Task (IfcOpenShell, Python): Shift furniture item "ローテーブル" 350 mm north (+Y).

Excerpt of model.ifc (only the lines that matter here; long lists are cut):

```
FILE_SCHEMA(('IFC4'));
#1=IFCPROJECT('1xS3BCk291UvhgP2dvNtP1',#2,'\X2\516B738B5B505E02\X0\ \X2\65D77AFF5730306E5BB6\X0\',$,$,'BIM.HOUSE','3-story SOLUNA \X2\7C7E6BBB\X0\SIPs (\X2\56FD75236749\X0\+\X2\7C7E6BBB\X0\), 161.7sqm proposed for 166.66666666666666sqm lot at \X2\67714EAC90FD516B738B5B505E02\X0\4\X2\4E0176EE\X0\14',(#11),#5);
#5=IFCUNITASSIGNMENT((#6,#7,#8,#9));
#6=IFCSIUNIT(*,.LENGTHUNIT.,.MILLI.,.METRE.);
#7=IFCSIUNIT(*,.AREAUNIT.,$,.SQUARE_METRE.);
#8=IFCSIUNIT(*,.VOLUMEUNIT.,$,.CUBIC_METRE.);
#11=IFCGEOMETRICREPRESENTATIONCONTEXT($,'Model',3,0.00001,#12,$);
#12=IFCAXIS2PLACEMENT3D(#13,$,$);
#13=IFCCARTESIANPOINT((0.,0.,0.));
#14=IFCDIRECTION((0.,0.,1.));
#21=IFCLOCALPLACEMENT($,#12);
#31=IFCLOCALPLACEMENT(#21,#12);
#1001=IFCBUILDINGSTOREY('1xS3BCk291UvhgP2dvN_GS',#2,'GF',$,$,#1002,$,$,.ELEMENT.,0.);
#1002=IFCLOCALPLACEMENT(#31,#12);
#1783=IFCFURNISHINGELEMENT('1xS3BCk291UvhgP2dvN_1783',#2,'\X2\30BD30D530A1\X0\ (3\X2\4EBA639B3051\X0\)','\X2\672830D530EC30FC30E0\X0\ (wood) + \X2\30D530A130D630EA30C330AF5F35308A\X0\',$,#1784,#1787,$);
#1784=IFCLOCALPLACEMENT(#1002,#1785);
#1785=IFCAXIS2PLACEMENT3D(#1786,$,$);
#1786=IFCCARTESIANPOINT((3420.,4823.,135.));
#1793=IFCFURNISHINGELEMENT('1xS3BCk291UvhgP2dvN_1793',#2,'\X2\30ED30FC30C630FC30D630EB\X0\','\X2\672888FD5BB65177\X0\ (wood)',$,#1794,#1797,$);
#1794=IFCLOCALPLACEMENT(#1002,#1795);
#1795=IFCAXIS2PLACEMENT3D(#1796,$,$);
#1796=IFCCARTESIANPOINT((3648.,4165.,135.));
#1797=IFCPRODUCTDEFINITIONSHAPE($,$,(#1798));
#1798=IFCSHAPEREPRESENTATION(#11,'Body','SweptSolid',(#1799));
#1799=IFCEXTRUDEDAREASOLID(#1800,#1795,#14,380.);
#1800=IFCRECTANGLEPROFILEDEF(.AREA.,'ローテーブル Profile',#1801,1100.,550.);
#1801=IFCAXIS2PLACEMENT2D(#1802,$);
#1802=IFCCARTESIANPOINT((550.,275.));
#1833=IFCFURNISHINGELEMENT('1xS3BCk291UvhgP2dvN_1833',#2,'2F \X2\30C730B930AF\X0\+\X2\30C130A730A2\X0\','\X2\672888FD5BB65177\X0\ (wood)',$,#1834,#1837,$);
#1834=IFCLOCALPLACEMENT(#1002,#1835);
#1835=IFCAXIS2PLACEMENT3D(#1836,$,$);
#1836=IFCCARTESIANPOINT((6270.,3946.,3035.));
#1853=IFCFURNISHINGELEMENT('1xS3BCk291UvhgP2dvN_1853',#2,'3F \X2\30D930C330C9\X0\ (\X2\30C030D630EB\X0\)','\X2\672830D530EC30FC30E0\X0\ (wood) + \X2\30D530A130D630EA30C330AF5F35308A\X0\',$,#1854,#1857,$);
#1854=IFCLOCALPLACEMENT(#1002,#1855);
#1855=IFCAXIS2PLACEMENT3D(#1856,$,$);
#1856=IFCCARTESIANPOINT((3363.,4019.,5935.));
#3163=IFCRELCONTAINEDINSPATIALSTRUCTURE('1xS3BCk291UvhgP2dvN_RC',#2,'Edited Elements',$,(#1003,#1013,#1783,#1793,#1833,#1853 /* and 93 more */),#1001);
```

```python
import ifcopenshell
import ifcopenshell.api.geometry
import ifcopenshell.util.placement

model = ifcopenshell.open("model.ifc")

item = model.by_id(1793)
matrix = ifcopenshell.util.placement.get_local_placement(item.ObjectPlacement)
matrix[1, 3] += 350.0
ifcopenshell.api.geometry.edit_object_placement(model, product=item, matrix=matrix, is_si=False)

print(ifcopenshell.util.placement.get_local_placement(item.ObjectPlacement).round(3) + 0.0)

model.write("model_updated.ifc")
```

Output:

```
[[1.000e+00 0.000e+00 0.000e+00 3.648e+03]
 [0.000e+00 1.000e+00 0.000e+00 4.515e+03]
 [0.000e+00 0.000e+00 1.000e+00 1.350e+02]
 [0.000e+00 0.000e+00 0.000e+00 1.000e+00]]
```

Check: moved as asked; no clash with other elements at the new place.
